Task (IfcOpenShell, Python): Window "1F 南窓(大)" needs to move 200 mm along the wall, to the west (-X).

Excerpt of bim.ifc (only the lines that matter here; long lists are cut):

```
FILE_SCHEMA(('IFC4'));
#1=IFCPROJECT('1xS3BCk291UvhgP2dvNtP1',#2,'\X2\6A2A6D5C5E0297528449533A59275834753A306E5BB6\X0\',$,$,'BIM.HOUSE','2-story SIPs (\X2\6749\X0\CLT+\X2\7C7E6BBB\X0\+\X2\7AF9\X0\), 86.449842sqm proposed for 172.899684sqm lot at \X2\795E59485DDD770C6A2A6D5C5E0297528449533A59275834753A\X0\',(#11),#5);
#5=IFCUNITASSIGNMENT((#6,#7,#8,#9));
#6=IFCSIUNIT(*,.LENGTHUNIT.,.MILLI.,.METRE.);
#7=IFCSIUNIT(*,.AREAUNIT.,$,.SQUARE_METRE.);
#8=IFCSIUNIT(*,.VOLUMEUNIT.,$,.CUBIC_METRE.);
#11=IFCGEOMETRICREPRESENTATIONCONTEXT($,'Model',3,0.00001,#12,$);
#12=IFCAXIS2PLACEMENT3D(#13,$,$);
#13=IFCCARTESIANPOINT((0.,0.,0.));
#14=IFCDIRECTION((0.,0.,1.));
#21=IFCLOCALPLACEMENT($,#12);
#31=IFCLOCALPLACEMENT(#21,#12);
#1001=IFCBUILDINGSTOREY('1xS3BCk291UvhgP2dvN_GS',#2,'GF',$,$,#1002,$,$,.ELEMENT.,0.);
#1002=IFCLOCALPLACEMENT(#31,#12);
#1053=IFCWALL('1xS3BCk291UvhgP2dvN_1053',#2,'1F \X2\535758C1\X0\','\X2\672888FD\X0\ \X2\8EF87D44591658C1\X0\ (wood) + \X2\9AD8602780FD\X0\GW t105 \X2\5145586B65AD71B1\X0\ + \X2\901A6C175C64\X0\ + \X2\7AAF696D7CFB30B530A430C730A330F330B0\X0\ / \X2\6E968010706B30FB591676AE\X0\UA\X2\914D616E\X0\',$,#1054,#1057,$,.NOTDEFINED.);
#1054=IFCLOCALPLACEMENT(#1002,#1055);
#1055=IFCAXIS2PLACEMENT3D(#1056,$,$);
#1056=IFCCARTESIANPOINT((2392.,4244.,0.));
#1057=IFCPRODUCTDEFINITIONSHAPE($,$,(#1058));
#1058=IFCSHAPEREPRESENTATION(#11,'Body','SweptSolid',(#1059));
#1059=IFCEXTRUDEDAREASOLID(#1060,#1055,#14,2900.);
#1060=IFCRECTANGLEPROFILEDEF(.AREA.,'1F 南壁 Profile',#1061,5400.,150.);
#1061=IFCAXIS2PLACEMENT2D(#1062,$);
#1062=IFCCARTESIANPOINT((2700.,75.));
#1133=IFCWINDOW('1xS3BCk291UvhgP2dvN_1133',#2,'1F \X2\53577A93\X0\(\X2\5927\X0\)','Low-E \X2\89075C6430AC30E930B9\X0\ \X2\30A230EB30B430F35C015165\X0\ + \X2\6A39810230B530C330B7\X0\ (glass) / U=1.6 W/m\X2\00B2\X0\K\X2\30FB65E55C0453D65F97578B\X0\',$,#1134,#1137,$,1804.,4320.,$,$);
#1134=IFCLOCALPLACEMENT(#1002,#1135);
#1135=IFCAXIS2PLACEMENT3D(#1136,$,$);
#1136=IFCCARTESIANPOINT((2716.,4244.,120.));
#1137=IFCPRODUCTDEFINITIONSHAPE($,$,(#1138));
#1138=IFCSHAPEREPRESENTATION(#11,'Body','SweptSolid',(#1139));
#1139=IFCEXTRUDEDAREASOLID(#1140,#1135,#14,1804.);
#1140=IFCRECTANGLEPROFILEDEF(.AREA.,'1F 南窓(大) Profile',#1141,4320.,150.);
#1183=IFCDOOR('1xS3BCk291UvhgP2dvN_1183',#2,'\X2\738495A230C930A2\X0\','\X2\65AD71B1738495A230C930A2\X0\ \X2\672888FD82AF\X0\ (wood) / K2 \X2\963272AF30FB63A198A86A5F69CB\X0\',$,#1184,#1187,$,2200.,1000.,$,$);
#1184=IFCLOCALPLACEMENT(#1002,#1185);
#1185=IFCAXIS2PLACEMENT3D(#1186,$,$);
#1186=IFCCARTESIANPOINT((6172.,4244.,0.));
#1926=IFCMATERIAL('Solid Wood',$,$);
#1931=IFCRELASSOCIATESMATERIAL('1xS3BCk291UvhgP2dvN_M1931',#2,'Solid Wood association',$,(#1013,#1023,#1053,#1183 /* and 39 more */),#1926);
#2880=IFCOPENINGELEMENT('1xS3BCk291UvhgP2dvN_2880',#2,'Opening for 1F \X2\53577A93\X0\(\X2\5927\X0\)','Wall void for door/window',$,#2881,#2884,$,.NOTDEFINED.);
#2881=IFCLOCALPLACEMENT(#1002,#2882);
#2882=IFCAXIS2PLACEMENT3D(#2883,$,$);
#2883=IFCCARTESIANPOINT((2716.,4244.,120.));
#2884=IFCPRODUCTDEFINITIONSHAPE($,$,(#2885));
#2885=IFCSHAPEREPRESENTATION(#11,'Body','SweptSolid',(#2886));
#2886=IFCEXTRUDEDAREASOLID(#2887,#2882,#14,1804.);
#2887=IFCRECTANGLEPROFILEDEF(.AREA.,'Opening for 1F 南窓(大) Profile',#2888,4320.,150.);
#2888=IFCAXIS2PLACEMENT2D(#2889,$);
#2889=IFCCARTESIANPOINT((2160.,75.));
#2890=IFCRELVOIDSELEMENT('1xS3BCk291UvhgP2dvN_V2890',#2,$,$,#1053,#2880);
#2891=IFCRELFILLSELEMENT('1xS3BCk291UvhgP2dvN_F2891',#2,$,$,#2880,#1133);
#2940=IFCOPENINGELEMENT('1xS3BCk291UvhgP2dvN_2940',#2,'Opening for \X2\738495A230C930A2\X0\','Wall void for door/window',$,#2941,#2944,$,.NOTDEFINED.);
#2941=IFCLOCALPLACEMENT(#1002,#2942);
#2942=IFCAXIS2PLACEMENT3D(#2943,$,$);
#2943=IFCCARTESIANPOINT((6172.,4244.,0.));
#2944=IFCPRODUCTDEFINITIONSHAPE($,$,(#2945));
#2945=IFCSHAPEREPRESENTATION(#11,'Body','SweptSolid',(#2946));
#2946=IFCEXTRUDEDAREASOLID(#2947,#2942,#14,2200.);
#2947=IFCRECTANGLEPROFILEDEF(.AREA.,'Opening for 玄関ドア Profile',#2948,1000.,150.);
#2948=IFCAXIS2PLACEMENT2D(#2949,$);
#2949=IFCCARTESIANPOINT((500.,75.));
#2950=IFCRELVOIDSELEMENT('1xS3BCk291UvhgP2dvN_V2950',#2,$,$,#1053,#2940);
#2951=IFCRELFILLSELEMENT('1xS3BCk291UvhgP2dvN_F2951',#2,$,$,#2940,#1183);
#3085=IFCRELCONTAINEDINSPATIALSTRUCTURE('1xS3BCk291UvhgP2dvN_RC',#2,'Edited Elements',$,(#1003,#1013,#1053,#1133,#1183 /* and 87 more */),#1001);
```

```python
import ifcopenshell
import ifcopenshell.api.geometry
import ifcopenshell.util.placement
import ifcopenshell.util.unit

model = ifcopenshell.open("bim.ifc")
unit_scale = ifcopenshell.util.unit.calculate_unit_scale(model)

window = model.by_guid("1xS3BCk291UvhgP2dvN_1133")
opening = window.FillsVoids[0].RelatingOpeningElement
wall = opening.VoidsElements[0].RelatingBuildingElement

wall_matrix = ifcopenshell.util.placement.get_local_placement(wall.ObjectPlacement)
shift = wall_matrix[:3, 0] * -0.2 / unit_scale
before = ifcopenshell.util.placement.get_local_placement(window.ObjectPlacement)[:3, 3].copy()

# The window is not placed relative to its opening, so move both.
for product in (opening, window):
    matrix = ifcopenshell.util.placement.get_local_placement(product.ObjectPlacement)
    matrix[:3, 3] += shift
    ifcopenshell.api.geometry.edit_object_placement(model, product=product, matrix=matrix, is_si=False)

after = ifcopenshell.util.placement.get_local_placement(window.ObjectPlacement)[:3, 3]
print("window moved by", (after - before).round(3) + 0.0)

model.write("bim-out.ifc")
```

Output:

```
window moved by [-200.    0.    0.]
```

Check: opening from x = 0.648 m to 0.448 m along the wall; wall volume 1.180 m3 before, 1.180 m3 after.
